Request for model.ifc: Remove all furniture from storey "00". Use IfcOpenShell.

First a look at what the model holds.

```python
import ifcopenshell
import ifcopenshell.util.element

model = ifcopenshell.open("model.ifc")
print(model.schema)
storey = next(s for s in model.by_type("IfcBuildingStorey") if s.Name == "00")
furniture = [e for e in ifcopenshell.util.element.get_decomposition(storey) if e.is_a("IfcFurnishingElement")]
seen = {}
for e in furniture:
    element_type = ifcopenshell.util.element.get_type(e)
    name = element_type.Name if element_type not in (None, e) else None
    seen[name] = seen.get(name, 0) + 1
for name, count in sorted(seen.items(), key=str):
    print(count, "x", name)
```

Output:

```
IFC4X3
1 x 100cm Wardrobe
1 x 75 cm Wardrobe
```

```python
import ifcopenshell
import ifcopenshell.api.root
import ifcopenshell.util.element

model = ifcopenshell.open("model.ifc")

storey = next(s for s in model.by_type("IfcBuildingStorey") if s.Name == "00")
furniture = [e for e in ifcopenshell.util.element.get_decomposition(storey) if e.is_a("IfcFurnishingElement")]

for e in furniture:
    ifcopenshell.api.root.remove_product(model, product=e)
print(len(furniture), "removed")

model.write("model-out.ifc")
```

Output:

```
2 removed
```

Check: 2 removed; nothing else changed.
